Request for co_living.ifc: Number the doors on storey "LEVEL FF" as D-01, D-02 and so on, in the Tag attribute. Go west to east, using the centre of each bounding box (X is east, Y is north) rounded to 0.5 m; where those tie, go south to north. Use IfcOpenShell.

First a look at what the model holds.

```python
import ifcopenshell
import ifcopenshell.util.element
import ifcopenshell.util.placement

model = ifcopenshell.open("co_living.ifc")
print(model.schema)
storey = next(s for s in model.by_type("IfcBuildingStorey") if s.Name == "LEVEL FF")
doors = [e for e in ifcopenshell.util.element.get_decomposition(storey) if e.is_a("IfcDoor")]
for e in sorted(doors, key=lambda e: e.id()):
    origin = ifcopenshell.util.placement.get_local_placement(e.ObjectPlacement)[:3, 3]
    print(e.id(), e.Tag, e.Name, origin.round(2) + 0.0, sep=" | ")
```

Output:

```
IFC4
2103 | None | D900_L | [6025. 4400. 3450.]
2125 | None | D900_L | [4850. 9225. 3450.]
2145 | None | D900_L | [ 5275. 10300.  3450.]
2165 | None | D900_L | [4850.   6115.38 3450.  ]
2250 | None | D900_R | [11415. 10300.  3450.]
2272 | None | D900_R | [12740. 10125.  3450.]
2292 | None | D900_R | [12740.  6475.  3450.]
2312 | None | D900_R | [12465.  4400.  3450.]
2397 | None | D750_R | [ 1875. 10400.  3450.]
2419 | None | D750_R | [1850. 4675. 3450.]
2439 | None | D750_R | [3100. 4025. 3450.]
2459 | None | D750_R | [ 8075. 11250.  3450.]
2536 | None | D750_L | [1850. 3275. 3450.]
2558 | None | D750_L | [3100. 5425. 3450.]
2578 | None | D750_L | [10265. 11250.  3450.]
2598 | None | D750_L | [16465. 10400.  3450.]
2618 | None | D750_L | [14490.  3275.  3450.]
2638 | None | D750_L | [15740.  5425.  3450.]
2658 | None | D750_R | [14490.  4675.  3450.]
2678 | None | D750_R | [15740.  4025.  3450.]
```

```python
import ifcopenshell
import ifcopenshell.geom
import ifcopenshell.util.element
import ifcopenshell.util.shape

model = ifcopenshell.open("co_living.ifc")
settings = ifcopenshell.geom.settings()
settings.set("use-world-coords", True)


def centre(element):
    shape = ifcopenshell.geom.create_shape(settings, element)
    return ifcopenshell.util.shape.get_bbox_centroid(shape.geometry)


storey = next(s for s in model.by_type("IfcBuildingStorey") if s.Name == "LEVEL FF")
doors = [e for e in ifcopenshell.util.element.get_decomposition(storey) if e.is_a("IfcDoor")]

# Insertion points can sit at a corner or the storey origin, so sort by the geometry (in metres).
centres = {e: centre(e) for e in doors}
doors.sort(key=lambda e: (round(centres[e][0] / 0.5), centres[e][1]))

for i, e in enumerate(doors, start=1):
    number = f"D-{i:02d}"
    e.Tag = number
    print(e.id(), number)

model.write("co_living-out.ifc")
```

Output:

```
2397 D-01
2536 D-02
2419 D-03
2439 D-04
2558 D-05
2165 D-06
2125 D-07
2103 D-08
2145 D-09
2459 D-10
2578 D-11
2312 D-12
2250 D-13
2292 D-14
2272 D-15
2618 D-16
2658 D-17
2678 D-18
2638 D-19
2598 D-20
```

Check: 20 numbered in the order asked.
